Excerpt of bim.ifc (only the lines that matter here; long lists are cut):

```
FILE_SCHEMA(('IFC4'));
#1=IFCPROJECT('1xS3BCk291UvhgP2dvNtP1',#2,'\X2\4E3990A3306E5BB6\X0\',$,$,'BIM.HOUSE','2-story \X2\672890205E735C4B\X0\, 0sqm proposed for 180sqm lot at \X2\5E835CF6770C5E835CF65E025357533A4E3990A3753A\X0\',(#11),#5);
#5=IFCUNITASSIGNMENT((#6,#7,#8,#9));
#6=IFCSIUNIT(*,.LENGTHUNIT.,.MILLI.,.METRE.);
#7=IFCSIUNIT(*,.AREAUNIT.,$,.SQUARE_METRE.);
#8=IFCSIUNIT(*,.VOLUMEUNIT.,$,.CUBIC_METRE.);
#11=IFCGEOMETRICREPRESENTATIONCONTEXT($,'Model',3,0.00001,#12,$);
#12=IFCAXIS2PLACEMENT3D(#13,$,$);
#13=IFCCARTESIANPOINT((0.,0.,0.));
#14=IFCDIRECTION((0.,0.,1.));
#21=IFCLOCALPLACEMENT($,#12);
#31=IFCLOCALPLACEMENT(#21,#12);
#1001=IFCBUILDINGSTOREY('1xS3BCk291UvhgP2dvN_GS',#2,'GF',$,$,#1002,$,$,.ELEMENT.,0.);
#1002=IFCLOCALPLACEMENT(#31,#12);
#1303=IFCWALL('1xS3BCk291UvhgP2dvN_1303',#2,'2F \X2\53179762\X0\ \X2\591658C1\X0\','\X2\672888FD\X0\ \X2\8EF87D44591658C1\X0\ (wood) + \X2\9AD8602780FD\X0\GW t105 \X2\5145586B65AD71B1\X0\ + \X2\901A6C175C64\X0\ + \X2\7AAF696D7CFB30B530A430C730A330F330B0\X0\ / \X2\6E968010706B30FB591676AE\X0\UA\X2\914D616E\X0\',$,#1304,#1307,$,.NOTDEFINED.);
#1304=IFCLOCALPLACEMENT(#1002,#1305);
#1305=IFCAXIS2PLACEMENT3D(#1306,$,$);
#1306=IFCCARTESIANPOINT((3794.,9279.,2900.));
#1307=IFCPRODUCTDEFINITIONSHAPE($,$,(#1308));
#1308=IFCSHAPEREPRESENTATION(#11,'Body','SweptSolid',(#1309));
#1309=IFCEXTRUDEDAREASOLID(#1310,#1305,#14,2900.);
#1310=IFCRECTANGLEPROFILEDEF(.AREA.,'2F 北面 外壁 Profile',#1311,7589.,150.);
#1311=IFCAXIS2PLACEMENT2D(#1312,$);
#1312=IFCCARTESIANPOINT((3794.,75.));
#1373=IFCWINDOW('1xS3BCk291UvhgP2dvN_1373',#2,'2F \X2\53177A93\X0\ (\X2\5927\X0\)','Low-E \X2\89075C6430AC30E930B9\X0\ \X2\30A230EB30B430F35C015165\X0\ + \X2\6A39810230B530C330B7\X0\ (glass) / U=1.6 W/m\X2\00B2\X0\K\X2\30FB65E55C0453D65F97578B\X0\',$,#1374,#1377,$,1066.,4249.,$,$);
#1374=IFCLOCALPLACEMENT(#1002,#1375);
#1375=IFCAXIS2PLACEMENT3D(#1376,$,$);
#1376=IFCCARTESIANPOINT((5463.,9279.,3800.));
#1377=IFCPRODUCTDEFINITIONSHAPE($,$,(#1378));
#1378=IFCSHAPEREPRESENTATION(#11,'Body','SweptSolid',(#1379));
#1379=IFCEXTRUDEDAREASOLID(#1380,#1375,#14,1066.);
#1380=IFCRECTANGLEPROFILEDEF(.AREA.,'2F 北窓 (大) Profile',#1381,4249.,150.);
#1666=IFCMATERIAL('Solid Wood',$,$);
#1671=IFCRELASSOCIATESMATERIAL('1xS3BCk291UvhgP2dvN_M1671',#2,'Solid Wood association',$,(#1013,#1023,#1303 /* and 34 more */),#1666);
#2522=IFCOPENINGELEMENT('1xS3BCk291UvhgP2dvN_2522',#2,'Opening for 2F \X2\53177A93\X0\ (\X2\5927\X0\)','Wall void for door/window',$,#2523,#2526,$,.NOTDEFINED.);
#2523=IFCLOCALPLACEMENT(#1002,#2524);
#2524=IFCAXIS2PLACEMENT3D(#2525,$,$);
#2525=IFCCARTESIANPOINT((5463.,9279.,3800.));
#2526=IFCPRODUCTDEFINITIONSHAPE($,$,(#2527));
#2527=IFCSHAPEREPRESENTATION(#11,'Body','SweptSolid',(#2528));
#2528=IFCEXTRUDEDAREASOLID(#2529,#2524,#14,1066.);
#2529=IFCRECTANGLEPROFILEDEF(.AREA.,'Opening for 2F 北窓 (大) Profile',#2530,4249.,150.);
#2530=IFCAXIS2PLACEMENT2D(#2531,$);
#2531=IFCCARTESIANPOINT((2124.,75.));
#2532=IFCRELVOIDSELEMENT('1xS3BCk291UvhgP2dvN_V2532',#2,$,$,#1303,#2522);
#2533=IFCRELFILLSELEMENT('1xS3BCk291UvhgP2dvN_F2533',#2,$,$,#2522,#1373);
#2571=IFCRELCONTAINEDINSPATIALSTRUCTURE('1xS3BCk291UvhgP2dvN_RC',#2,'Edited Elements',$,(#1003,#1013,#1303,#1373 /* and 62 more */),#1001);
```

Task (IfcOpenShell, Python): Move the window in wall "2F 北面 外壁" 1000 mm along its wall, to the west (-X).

```python
import ifcopenshell
import ifcopenshell.api.geometry
import ifcopenshell.util.placement
import ifcopenshell.util.unit

model = ifcopenshell.open("bim.ifc")
unit_scale = ifcopenshell.util.unit.calculate_unit_scale(model)

window = model.by_id(1373)
opening = window.FillsVoids[0].RelatingOpeningElement
wall = opening.VoidsElements[0].RelatingBuildingElement

wall_matrix = ifcopenshell.util.placement.get_local_placement(wall.ObjectPlacement)
shift = wall_matrix[:3, 0] * -1 / unit_scale
before = ifcopenshell.util.placement.get_local_placement(window.ObjectPlacement)[:3, 3].copy()

# The window is not placed relative to its opening, so move both.
for product in (opening, window):
    matrix = ifcopenshell.util.placement.get_local_placement(product.ObjectPlacement)
    matrix[:3, 3] += shift
    ifcopenshell.api.geometry.edit_object_placement(model, product=product, matrix=matrix, is_si=False)

after = ifcopenshell.util.placement.get_local_placement(window.ObjectPlacement)[:3, 3]
print("window moved by", (after - before).round(3) + 0.0)

model.write("bim_v2.ifc")
```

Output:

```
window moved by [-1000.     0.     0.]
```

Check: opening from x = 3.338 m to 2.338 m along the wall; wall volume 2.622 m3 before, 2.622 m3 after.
